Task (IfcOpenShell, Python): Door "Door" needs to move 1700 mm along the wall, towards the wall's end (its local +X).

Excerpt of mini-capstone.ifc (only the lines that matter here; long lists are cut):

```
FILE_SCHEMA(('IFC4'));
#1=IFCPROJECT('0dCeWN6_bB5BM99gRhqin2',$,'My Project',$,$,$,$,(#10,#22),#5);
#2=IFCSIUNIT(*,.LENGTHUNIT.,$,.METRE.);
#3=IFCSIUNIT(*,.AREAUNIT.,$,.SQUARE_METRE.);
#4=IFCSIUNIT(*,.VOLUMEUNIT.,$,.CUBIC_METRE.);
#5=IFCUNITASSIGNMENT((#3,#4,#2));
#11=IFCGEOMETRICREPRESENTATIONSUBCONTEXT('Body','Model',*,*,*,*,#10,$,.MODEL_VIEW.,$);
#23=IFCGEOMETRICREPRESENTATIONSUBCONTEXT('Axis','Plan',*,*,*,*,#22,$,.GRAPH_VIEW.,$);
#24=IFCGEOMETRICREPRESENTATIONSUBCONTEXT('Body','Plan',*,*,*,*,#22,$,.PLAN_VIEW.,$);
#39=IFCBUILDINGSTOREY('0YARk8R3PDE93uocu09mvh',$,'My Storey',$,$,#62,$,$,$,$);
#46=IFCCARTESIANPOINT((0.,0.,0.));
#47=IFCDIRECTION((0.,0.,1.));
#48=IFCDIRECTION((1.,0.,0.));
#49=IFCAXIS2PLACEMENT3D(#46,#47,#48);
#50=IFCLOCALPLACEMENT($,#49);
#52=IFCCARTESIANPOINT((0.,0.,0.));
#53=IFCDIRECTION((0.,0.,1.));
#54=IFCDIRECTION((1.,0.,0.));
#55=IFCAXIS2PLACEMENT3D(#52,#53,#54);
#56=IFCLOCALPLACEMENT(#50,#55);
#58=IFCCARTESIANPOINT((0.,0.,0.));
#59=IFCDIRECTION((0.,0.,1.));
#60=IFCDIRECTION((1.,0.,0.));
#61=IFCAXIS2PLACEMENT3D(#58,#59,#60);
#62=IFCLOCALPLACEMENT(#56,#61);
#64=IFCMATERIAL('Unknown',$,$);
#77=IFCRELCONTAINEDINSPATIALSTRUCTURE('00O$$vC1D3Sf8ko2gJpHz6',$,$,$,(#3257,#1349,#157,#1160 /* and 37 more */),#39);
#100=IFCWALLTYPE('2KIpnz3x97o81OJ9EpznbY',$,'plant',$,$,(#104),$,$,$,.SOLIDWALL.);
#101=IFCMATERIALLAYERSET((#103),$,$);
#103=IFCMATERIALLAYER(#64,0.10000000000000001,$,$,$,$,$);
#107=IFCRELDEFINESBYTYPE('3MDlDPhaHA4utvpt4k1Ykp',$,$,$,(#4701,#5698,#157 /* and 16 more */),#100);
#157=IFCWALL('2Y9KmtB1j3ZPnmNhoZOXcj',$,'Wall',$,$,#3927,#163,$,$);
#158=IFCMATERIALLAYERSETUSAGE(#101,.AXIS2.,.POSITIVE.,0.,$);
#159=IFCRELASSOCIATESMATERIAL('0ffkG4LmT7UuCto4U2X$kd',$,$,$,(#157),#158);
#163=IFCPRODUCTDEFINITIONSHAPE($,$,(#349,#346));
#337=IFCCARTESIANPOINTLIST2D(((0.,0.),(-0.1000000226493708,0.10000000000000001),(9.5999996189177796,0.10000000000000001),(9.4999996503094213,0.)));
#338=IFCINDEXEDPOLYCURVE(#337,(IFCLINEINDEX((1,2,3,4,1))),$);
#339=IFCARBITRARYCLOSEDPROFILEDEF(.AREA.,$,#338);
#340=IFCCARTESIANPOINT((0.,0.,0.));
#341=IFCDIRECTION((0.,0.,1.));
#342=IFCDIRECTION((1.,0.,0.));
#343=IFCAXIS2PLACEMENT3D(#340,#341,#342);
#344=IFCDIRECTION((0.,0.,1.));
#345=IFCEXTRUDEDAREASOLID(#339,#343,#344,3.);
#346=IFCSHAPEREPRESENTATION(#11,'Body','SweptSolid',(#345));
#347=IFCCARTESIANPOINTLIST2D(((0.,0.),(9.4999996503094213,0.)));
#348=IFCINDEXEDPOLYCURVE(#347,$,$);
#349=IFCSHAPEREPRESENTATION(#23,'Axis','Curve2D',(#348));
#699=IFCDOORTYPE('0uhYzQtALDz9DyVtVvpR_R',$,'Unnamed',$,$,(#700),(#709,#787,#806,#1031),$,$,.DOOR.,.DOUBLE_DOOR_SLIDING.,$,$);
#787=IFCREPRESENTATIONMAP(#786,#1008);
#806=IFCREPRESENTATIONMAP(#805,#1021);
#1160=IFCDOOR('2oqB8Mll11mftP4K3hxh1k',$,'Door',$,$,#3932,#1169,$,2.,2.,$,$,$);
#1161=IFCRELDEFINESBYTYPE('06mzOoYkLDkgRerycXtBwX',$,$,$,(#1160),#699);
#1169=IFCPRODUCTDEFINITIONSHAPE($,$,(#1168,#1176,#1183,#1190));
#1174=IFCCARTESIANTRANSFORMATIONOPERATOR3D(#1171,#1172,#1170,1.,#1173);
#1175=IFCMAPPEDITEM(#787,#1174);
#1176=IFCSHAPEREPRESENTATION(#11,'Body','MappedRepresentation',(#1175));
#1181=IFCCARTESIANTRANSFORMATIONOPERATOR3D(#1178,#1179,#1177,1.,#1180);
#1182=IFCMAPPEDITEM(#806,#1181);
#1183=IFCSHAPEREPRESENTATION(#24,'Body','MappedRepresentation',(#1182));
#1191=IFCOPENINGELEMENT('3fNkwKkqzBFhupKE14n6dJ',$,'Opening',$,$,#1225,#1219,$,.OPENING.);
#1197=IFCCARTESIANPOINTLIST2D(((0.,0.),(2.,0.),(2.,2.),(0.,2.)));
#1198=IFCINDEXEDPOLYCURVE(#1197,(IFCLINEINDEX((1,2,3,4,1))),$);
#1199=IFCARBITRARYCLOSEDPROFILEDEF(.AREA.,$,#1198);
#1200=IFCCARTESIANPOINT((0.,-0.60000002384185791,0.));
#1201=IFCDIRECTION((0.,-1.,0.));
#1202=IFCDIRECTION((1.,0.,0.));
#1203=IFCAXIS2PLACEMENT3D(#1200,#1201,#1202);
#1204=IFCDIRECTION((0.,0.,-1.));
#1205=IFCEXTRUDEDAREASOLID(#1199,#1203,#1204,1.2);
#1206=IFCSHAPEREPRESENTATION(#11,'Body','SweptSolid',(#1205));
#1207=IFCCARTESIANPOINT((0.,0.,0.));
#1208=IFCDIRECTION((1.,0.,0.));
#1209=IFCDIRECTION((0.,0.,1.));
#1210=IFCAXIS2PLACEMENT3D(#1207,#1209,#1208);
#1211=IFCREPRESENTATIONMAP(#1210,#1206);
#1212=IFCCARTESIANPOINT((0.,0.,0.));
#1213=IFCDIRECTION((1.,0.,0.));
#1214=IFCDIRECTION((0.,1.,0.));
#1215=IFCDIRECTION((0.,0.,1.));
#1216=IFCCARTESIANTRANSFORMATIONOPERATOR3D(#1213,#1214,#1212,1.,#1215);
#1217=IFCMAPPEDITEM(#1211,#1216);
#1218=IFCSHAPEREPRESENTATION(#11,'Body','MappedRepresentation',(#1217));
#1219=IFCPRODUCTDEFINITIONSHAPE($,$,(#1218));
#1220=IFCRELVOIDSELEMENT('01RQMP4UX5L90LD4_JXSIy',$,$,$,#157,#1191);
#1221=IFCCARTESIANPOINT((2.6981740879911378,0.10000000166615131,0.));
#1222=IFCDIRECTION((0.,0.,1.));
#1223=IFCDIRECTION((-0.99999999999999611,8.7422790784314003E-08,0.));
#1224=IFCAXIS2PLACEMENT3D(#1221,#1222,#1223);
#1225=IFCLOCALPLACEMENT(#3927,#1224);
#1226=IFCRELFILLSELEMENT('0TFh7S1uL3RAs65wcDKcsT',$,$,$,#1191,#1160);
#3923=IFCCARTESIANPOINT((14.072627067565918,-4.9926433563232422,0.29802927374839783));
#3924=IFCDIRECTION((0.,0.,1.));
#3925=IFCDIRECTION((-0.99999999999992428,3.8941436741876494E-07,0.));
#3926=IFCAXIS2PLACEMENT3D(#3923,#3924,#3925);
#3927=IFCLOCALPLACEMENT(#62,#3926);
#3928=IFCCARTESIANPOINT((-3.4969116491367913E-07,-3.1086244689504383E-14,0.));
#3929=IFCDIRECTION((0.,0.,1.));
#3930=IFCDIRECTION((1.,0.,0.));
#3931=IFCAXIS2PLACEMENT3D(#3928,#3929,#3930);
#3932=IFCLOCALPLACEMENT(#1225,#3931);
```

```python
import ifcopenshell
import ifcopenshell.api.geometry
import ifcopenshell.util.placement

model = ifcopenshell.open("mini-capstone.ifc")

door = model.by_id(1160)
opening = door.FillsVoids[0].RelatingOpeningElement
wall = opening.VoidsElements[0].RelatingBuildingElement

wall_matrix = ifcopenshell.util.placement.get_local_placement(wall.ObjectPlacement)
shift = wall_matrix[:3, 0] * 1.7
before = ifcopenshell.util.placement.get_local_placement(door.ObjectPlacement)[:3, 3].copy()

# The door is placed relative to its opening, so it follows when the opening moves.
matrix = ifcopenshell.util.placement.get_local_placement(opening.ObjectPlacement)
matrix[:3, 3] += shift
ifcopenshell.api.geometry.edit_object_placement(
    model, product=opening, matrix=matrix, is_si=False, should_transform_children=True
)

after = ifcopenshell.util.placement.get_local_placement(door.ObjectPlacement)[:3, 3]
print("door moved by", (after - before).round(3) + 0.0)

model.write("mini-capstone_v2.ifc")
```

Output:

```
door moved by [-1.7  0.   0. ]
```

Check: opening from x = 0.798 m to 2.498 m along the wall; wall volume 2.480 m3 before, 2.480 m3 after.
